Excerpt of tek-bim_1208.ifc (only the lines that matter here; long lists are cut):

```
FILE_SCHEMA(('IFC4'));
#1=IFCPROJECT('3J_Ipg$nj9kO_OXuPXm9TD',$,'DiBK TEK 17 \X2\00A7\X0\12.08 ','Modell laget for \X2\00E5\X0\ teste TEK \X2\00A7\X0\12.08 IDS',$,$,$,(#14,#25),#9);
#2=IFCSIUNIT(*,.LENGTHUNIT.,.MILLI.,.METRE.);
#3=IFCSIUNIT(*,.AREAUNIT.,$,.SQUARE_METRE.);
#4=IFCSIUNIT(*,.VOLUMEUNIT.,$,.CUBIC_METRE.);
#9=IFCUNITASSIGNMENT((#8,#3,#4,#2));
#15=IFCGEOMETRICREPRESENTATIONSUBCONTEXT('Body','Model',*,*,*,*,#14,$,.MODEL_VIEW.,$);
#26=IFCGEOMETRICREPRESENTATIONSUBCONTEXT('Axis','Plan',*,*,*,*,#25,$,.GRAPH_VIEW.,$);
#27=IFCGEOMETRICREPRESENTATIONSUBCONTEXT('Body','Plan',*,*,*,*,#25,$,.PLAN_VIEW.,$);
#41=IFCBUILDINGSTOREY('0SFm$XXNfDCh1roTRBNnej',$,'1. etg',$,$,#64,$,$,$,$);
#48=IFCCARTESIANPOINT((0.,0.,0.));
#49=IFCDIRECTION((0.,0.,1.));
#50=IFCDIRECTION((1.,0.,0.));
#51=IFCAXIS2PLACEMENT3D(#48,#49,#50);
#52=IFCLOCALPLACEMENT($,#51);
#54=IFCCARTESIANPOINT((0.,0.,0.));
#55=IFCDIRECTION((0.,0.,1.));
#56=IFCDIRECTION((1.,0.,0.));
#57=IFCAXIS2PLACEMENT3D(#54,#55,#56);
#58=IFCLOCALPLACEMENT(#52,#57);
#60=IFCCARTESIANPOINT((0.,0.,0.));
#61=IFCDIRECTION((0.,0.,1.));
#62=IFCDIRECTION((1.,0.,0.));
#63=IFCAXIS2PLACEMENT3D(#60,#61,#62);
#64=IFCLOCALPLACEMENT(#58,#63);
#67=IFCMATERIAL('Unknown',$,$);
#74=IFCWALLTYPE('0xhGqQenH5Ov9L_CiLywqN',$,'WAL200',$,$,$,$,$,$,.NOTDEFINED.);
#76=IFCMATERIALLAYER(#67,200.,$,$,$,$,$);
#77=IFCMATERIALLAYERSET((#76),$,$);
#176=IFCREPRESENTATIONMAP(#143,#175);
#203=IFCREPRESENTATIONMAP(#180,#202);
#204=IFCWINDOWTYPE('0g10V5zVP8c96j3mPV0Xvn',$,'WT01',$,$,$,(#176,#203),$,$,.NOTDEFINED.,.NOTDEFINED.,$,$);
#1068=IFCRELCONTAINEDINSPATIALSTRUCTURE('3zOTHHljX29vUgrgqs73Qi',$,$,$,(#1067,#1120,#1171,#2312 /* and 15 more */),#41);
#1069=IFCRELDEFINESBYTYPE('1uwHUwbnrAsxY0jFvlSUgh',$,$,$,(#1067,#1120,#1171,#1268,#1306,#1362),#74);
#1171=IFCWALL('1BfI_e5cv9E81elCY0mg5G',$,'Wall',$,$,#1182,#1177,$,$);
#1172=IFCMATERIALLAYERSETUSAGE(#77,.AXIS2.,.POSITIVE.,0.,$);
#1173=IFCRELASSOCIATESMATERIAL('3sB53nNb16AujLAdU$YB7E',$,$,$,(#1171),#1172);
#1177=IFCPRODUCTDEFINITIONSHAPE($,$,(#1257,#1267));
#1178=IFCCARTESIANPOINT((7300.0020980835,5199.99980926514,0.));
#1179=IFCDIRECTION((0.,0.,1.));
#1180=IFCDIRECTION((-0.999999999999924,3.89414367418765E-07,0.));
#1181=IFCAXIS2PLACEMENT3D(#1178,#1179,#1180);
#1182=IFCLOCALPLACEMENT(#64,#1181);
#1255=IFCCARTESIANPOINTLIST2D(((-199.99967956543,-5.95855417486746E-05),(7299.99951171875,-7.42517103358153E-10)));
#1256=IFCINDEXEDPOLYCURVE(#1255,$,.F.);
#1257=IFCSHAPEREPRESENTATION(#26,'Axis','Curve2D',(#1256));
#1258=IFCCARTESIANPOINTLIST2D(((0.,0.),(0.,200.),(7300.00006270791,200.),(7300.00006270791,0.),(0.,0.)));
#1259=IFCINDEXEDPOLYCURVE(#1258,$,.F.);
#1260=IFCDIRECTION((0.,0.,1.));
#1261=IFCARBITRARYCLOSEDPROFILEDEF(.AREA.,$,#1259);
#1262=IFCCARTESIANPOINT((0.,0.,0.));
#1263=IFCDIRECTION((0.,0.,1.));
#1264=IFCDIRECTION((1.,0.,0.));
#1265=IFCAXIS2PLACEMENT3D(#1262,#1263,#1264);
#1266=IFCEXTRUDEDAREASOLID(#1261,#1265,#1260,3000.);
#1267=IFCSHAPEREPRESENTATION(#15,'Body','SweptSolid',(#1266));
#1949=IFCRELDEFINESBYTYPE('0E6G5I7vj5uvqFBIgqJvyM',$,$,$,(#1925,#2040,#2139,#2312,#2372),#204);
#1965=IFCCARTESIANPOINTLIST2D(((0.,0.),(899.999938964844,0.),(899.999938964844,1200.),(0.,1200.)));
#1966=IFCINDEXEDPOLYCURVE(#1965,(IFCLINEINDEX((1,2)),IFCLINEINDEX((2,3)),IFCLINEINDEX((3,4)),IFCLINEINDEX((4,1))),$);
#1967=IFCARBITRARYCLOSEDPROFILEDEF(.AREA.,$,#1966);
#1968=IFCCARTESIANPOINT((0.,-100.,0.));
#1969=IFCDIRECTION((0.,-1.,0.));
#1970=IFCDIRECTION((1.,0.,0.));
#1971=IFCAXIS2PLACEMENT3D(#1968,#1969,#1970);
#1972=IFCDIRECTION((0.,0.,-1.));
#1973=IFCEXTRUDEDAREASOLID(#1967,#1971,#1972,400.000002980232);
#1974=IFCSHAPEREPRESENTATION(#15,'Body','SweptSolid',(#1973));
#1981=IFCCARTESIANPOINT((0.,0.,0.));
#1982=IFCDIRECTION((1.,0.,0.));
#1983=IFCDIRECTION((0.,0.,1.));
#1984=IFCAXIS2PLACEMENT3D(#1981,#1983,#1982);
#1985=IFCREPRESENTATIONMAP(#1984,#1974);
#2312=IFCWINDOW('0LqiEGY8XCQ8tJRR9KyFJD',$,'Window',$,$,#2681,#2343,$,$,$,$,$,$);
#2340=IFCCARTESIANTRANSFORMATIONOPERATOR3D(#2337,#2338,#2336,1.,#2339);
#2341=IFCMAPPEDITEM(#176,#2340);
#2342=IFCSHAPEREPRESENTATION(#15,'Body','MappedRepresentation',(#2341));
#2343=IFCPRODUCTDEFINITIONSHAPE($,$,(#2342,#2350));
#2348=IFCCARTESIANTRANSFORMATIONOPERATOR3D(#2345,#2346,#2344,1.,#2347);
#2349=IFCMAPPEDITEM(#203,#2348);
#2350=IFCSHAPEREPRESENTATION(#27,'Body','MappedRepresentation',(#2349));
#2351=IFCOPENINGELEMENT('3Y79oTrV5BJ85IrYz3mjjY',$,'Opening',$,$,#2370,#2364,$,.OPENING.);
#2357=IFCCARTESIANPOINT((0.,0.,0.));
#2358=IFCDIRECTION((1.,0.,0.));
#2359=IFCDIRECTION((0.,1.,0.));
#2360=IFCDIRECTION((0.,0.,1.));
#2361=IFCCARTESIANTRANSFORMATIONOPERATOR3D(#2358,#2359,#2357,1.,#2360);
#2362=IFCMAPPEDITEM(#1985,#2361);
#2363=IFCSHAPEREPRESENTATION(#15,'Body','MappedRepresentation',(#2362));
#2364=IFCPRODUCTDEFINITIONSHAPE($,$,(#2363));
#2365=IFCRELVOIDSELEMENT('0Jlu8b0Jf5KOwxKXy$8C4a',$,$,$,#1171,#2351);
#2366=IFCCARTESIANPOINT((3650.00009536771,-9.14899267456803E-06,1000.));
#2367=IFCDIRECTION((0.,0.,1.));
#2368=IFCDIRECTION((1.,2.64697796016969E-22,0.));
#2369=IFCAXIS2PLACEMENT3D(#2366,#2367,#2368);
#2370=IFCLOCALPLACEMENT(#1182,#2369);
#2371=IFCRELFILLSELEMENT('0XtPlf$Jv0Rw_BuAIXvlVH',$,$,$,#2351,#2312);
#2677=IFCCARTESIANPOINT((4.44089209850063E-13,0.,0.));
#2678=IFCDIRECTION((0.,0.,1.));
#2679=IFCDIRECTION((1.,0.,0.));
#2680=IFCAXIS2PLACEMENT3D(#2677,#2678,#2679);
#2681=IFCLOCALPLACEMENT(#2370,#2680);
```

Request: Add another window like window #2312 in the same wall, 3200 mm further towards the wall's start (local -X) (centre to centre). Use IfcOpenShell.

```python
import ifcopenshell
import ifcopenshell.api.feature
import ifcopenshell.api.geometry
import ifcopenshell.api.root
import ifcopenshell.geom
import ifcopenshell.util.element
import ifcopenshell.util.placement
import ifcopenshell.util.shape

model = ifcopenshell.open("tek-bim_1208.ifc")
settings = ifcopenshell.geom.settings()


def volume(element):
    """Net volume in cubic metres, openings subtracted."""
    shape = ifcopenshell.geom.create_shape(settings, element)
    return ifcopenshell.util.shape.get_volume(shape.geometry)


window = model.by_id(2312)
opening = window.FillsVoids[0].RelatingOpeningElement
wall = opening.VoidsElements[0].RelatingBuildingElement
before = volume(wall)
shift = ifcopenshell.util.placement.get_local_placement(wall.ObjectPlacement)[:3, 0] * -3200.0

# copy_class copies the void relationship, type, container and properties, but no geometry.
new_opening = ifcopenshell.api.root.copy_class(model, product=opening)
new_opening.Representation = ifcopenshell.util.element.copy_deep(
    model, opening.Representation, exclude=["IfcGeometricRepresentationContext", "IfcRepresentationMap"]
)
new_window = ifcopenshell.api.root.copy_class(model, product=window)
new_window.Representation = ifcopenshell.util.element.copy_deep(
    model, window.Representation, exclude=["IfcGeometricRepresentationContext", "IfcRepresentationMap"]
)
ifcopenshell.api.feature.add_filling(model, opening=new_opening, element=new_window)

for old, new in ((opening, new_opening), (window, new_window)):
    matrix = ifcopenshell.util.placement.get_local_placement(old.ObjectPlacement)
    matrix[:3, 3] += shift
    ifcopenshell.api.geometry.edit_object_placement(model, product=new, matrix=matrix, is_si=False)

after = volume(wall)

print(f"wall volume {before:.3f} -> {after:.3f} m3")

model.write("tek-bim_1208_edited.ifc")
```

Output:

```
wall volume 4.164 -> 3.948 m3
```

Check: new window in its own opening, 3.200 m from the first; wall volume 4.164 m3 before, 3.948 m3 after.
